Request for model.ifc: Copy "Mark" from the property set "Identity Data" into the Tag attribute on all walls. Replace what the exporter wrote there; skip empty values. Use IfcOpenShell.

First a look at what the model holds.

```python
import ifcopenshell
import ifcopenshell.util.element

model = ifcopenshell.open("model.ifc")
print(model.schema)
walls = model.by_type("IfcWall")
print(len(walls), "walls")
for e in walls[:8]:
    source = ifcopenshell.util.element.get_pset(e, "Identity Data", "Mark")
    target = e.Tag
    print(e.id(), repr(source), repr(target), sep=" | ")
```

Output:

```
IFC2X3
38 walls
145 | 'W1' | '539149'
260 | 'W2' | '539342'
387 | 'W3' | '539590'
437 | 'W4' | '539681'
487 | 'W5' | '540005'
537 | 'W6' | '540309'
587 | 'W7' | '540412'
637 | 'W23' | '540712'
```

```python
import ifcopenshell
import ifcopenshell.util.element

model = ifcopenshell.open("model.ifc")

count = 0
for e in model.by_type("IfcWall"):
    value = ifcopenshell.util.element.get_pset(e, "Identity Data", "Mark")
    current = e.Tag
    if not value or not value.strip() or current == value:
        continue
    e.Tag = value
    count += 1

print(count, "walls updated")

model.write("model_updated.ifc")
```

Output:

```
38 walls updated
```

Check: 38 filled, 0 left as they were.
